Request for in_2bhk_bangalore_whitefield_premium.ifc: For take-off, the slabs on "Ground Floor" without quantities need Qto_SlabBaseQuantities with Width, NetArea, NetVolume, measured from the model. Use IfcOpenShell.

First a look at what the model holds.

```python
import ifcopenshell
import ifcopenshell.util.element
import ifcopenshell.util.unit

model = ifcopenshell.open("in_2bhk_bangalore_whitefield_premium.ifc")
print(model.schema)
for unit_type in ("LENGTHUNIT", "AREAUNIT", "VOLUMEUNIT"):
    print(unit_type, ifcopenshell.util.unit.calculate_unit_scale(model, unit_type))
storey = next(s for s in model.by_type("IfcBuildingStorey") if s.Name == "Ground Floor")
slabs = [e for e in ifcopenshell.util.element.get_decomposition(storey) if e.is_a("IfcSlab")]
for e in sorted(slabs, key=lambda e: e.id()):
    print(e.id(), e.is_a(), e.Name, list(ifcopenshell.util.element.get_psets(e, qtos_only=True)), sep=" | ")
```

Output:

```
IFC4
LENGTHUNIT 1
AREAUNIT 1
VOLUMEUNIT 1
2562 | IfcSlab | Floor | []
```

```python
import ifcopenshell
import ifcopenshell.api.pset
import ifcopenshell.geom
import ifcopenshell.util.element
import ifcopenshell.util.shape
import ifcopenshell.util.unit

model = ifcopenshell.open("in_2bhk_bangalore_whitefield_premium.ifc")
unit_scale = ifcopenshell.util.unit.calculate_unit_scale(model)
area_scale = ifcopenshell.util.unit.calculate_unit_scale(model, "AREAUNIT")
volume_scale = ifcopenshell.util.unit.calculate_unit_scale(model, "VOLUMEUNIT")
settings = ifcopenshell.geom.settings()

storey = next(s for s in model.by_type("IfcBuildingStorey") if s.Name == "Ground Floor")
slabs = [e for e in ifcopenshell.util.element.get_decomposition(storey) if e.is_a("IfcSlab")]

for e in sorted(slabs, key=lambda e: e.id()):
    if ifcopenshell.util.element.get_psets(e, qtos_only=True, should_inherit=False):
        continue
    # Geometry comes back in metres, in the element's own axes.
    shape = ifcopenshell.geom.create_shape(settings, e)
    values = {
        "Width": ifcopenshell.util.shape.get_z(shape.geometry) / unit_scale,
        "NetArea": ifcopenshell.util.shape.get_footprint_area(shape.geometry) / area_scale,
        "NetVolume": ifcopenshell.util.shape.get_volume(shape.geometry) / volume_scale,
    }
    qto = ifcopenshell.api.pset.add_qto(model, product=e, name="Qto_SlabBaseQuantities")
    ifcopenshell.api.pset.edit_qto(model, qto=qto, properties=values)
    print(e.id(), {k: round(v, 3) for k, v in values.items()})

model.write("in_2bhk_bangalore_whitefield_premium-out.ifc")
```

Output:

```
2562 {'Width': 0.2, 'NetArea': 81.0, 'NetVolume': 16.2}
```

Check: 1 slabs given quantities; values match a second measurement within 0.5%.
